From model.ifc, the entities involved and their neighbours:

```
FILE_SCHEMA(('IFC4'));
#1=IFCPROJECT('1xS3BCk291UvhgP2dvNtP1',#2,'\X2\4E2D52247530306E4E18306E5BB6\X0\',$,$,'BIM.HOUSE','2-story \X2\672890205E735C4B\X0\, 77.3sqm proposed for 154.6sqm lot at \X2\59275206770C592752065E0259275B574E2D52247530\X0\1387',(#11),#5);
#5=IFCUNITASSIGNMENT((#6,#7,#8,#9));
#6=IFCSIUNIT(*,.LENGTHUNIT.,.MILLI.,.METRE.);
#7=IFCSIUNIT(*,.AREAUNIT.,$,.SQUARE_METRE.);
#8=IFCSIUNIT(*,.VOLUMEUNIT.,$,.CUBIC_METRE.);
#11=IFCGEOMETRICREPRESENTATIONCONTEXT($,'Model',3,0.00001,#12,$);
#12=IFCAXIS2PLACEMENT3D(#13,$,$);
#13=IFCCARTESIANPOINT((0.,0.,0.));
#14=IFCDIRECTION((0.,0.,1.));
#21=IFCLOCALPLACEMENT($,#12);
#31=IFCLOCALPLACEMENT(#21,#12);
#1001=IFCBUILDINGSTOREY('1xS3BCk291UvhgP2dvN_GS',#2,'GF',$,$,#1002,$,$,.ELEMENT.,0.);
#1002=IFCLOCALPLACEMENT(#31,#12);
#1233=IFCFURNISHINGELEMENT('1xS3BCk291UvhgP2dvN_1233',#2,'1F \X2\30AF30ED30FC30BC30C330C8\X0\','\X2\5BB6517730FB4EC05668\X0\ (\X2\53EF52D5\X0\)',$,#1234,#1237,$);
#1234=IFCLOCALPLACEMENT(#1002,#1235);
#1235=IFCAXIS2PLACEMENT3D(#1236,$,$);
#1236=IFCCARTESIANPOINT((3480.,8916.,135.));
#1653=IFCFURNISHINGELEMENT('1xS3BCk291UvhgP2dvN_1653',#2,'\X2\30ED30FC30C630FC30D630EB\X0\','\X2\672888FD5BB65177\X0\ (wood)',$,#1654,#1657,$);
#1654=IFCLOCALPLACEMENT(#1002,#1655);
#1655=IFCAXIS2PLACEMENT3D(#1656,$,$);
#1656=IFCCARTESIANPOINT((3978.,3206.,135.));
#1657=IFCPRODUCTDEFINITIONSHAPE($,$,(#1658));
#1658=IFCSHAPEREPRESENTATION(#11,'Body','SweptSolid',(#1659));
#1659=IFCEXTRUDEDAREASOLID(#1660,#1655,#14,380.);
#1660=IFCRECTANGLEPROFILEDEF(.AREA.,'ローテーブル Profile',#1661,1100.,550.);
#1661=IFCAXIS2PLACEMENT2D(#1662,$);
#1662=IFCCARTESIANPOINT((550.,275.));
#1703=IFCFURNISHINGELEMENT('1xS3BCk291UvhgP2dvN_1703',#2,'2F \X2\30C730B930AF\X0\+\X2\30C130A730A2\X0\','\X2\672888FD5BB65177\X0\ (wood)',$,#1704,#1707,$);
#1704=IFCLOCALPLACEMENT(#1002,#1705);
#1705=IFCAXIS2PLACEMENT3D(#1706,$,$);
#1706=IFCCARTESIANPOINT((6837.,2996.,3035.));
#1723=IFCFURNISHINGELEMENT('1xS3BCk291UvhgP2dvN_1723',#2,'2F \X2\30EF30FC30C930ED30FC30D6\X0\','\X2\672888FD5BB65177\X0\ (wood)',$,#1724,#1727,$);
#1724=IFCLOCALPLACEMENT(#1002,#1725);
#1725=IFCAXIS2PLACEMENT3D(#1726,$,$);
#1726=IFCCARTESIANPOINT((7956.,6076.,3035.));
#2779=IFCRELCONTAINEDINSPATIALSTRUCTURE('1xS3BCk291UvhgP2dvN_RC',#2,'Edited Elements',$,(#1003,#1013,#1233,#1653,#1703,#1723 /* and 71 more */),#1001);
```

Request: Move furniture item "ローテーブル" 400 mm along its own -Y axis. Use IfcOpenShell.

```python
import ifcopenshell
import ifcopenshell.api.geometry
import ifcopenshell.util.placement

model = ifcopenshell.open("model.ifc")

item = model.by_guid("1xS3BCk291UvhgP2dvN_1653")
matrix = ifcopenshell.util.placement.get_local_placement(item.ObjectPlacement)
matrix[:3, 3] -= matrix[:3, 1] * 400.0
ifcopenshell.api.geometry.edit_object_placement(model, product=item, matrix=matrix, is_si=False)

print(ifcopenshell.util.placement.get_local_placement(item.ObjectPlacement).round(3) + 0.0)

model.write("model-out.ifc")
```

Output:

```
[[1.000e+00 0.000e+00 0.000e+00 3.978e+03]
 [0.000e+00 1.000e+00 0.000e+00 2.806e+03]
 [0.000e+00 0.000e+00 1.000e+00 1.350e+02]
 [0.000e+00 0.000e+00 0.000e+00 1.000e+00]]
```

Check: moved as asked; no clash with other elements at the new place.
